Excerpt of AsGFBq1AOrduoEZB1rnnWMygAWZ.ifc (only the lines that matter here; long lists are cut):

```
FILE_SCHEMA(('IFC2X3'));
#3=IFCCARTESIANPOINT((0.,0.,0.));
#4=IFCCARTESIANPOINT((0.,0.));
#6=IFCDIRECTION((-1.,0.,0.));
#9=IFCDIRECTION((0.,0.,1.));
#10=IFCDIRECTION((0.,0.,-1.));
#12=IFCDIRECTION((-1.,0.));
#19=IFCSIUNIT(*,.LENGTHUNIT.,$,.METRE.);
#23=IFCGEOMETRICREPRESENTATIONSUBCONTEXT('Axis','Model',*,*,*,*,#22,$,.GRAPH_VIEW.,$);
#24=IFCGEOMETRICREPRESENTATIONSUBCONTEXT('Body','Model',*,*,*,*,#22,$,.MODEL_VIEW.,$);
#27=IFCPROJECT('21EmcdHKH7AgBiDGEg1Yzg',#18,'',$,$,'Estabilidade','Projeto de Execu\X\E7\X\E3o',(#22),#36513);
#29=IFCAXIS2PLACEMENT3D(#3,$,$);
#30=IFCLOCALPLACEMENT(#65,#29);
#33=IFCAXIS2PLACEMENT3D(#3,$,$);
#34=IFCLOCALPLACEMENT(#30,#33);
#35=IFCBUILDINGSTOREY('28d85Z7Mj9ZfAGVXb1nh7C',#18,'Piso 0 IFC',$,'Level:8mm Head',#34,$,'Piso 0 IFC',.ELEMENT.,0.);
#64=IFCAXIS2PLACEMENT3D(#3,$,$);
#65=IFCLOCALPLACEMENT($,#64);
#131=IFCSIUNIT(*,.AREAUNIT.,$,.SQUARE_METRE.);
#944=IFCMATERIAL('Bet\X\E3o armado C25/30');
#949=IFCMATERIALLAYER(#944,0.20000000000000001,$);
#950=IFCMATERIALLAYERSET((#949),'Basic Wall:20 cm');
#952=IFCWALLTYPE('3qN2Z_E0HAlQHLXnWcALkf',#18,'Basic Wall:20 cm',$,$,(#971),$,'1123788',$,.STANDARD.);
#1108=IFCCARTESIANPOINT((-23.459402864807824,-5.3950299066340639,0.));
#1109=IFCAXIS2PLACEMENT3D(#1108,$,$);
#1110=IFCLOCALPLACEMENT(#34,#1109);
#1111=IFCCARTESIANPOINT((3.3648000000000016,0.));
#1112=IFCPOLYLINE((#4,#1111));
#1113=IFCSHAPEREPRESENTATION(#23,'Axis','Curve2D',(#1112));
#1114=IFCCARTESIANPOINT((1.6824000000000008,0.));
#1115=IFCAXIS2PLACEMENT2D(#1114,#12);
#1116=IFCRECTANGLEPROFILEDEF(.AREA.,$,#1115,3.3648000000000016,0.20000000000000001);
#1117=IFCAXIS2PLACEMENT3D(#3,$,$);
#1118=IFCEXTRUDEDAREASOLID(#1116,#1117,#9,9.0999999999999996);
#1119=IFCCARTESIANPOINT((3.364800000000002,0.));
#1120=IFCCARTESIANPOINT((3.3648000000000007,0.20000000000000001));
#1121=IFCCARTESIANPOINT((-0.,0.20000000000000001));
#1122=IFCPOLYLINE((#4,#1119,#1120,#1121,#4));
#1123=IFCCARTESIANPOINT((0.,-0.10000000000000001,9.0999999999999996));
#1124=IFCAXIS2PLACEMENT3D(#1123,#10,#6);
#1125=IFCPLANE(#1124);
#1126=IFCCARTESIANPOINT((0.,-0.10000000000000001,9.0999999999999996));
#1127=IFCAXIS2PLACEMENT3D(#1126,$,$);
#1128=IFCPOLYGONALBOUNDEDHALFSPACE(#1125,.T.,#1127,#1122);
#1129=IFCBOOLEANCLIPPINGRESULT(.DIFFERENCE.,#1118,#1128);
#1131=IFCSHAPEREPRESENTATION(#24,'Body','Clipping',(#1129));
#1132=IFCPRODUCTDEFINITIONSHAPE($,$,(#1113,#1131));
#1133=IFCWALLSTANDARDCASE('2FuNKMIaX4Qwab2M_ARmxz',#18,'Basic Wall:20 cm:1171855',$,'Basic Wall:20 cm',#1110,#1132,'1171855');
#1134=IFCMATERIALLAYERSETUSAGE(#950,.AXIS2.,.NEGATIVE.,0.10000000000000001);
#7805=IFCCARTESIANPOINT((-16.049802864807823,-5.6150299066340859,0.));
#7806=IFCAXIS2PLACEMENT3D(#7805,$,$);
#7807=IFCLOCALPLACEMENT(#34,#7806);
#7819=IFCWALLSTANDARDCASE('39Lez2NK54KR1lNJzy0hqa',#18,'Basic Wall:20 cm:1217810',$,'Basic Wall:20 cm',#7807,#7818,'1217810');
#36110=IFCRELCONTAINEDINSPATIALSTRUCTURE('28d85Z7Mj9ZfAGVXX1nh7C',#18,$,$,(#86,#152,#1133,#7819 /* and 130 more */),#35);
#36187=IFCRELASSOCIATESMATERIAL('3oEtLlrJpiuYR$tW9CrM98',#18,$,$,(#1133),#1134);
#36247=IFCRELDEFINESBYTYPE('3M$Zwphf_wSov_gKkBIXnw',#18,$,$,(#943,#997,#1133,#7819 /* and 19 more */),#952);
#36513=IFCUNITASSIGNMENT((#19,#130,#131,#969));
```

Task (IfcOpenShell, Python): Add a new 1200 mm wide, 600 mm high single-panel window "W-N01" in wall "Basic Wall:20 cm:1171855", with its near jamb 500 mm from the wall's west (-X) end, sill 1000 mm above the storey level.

```python
import numpy as np
import ifcopenshell
import ifcopenshell.api.feature
import ifcopenshell.api.geometry
import ifcopenshell.api.root
import ifcopenshell.api.spatial
import ifcopenshell.api.type
import ifcopenshell.geom
import ifcopenshell.util.element
import ifcopenshell.util.placement
import ifcopenshell.util.representation
import ifcopenshell.util.shape
import ifcopenshell.util.unit

model = ifcopenshell.open("AsGFBq1AOrduoEZB1rnnWMygAWZ.ifc")
unit_scale = ifcopenshell.util.unit.calculate_unit_scale(model)
settings = ifcopenshell.geom.settings()


def volume(element):
    """Net volume in cubic metres, openings subtracted."""
    shape = ifcopenshell.geom.create_shape(settings, element)
    return ifcopenshell.util.shape.get_volume(shape.geometry)


wall = model.by_guid("2FuNKMIaX4Qwab2M_ARmxz")
storey = ifcopenshell.util.element.get_container(wall, ifc_class="IfcBuildingStorey")
context = ifcopenshell.util.representation.get_context(model, "Model", "Body", "MODEL_VIEW")
before = volume(wall)

width, height, from_end, sill = 1.2, 0.6, 0.5, 1  # metres

# The wall runs along its own X axis, and the end named is its -X end.
wall_shape = ifcopenshell.geom.create_shape(settings, wall)
x, y, z = ifcopenshell.util.shape.get_vertices(wall_shape.geometry).T
start = x.min() + from_end
face, thickness = float(y.min()), float(y.max() - y.min())
wall_matrix = ifcopenshell.util.placement.get_local_placement(wall.ObjectPlacement)
level = ifcopenshell.util.placement.get_local_placement(storey.ObjectPlacement)[2, 3]


def in_wall(x, y):
    """Placement at x, y metres in the wall's axes, at sill height."""
    matrix = wall_matrix.copy()
    matrix[:, 3] = wall_matrix @ np.array([x / unit_scale, y / unit_scale, 0.0, 1.0])
    matrix[2, 3] = level + sill / unit_scale
    return matrix


# Opening: a box that overshoots both wall faces by 50 mm.
opening = ifcopenshell.api.root.create_entity(model, ifc_class="IfcOpeningElement")
box = ifcopenshell.api.geometry.add_wall_representation(
    model, context=context, length=width, height=height, thickness=thickness + 0.1
)
ifcopenshell.api.geometry.assign_representation(model, product=opening, representation=box)
ifcopenshell.api.geometry.edit_object_placement(model, product=opening, matrix=in_wall(start, face - 0.05), is_si=False)
ifcopenshell.api.feature.add_feature(model, feature=opening, element=wall)

window = ifcopenshell.api.root.create_entity(model, ifc_class="IfcWindow", name="W-N01")
window.OverallWidth, window.OverallHeight = width / unit_scale, height / unit_scale
body = ifcopenshell.api.geometry.add_window_representation(
    model,
    context=context,
    overall_width=window.OverallWidth,
    overall_height=window.OverallHeight,
    partition_type="SINGLE_PANEL",
)
ifcopenshell.api.geometry.assign_representation(model, product=window, representation=body)
ifcopenshell.api.spatial.assign_container(model, products=[window], relating_structure=storey)
fills = ifcopenshell.api.feature.add_filling(model, opening=opening, element=window)
fills.OwnerHistory = window.OwnerHistory  # required in IFC2X3

# IFC2X3 keeps the operation on the window style.
style = ifcopenshell.api.root.create_entity(model, ifc_class="IfcWindowStyle", name="W-N01")
style.OperationType, style.ConstructionType = "SINGLE_PANEL", "NOTDEFINED"
style.ParameterTakesPrecedence = style.Sizeable = False
ifcopenshell.api.type.assign_type(model, related_objects=[window], relating_type=style)

# Centre the window in the wall's thickness.
ifcopenshell.api.geometry.edit_object_placement(model, product=window, matrix=in_wall(start, face), is_si=False)
window_shape = ifcopenshell.geom.create_shape(settings, window)
depth = ifcopenshell.util.shape.get_vertices(window_shape.geometry)[:, 1]
offset = face + thickness / 2 - (depth.min() + depth.max()) / 2
ifcopenshell.api.geometry.edit_object_placement(model, product=window, matrix=in_wall(start, offset), is_si=False)

after = volume(wall)

print(f"wall volume {before:.3f} -> {after:.3f} m3")

model.write("AsGFBq1AOrduoEZB1rnnWMygAWZ_edited.ifc")
```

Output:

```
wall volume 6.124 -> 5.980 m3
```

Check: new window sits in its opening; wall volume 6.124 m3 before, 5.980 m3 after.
